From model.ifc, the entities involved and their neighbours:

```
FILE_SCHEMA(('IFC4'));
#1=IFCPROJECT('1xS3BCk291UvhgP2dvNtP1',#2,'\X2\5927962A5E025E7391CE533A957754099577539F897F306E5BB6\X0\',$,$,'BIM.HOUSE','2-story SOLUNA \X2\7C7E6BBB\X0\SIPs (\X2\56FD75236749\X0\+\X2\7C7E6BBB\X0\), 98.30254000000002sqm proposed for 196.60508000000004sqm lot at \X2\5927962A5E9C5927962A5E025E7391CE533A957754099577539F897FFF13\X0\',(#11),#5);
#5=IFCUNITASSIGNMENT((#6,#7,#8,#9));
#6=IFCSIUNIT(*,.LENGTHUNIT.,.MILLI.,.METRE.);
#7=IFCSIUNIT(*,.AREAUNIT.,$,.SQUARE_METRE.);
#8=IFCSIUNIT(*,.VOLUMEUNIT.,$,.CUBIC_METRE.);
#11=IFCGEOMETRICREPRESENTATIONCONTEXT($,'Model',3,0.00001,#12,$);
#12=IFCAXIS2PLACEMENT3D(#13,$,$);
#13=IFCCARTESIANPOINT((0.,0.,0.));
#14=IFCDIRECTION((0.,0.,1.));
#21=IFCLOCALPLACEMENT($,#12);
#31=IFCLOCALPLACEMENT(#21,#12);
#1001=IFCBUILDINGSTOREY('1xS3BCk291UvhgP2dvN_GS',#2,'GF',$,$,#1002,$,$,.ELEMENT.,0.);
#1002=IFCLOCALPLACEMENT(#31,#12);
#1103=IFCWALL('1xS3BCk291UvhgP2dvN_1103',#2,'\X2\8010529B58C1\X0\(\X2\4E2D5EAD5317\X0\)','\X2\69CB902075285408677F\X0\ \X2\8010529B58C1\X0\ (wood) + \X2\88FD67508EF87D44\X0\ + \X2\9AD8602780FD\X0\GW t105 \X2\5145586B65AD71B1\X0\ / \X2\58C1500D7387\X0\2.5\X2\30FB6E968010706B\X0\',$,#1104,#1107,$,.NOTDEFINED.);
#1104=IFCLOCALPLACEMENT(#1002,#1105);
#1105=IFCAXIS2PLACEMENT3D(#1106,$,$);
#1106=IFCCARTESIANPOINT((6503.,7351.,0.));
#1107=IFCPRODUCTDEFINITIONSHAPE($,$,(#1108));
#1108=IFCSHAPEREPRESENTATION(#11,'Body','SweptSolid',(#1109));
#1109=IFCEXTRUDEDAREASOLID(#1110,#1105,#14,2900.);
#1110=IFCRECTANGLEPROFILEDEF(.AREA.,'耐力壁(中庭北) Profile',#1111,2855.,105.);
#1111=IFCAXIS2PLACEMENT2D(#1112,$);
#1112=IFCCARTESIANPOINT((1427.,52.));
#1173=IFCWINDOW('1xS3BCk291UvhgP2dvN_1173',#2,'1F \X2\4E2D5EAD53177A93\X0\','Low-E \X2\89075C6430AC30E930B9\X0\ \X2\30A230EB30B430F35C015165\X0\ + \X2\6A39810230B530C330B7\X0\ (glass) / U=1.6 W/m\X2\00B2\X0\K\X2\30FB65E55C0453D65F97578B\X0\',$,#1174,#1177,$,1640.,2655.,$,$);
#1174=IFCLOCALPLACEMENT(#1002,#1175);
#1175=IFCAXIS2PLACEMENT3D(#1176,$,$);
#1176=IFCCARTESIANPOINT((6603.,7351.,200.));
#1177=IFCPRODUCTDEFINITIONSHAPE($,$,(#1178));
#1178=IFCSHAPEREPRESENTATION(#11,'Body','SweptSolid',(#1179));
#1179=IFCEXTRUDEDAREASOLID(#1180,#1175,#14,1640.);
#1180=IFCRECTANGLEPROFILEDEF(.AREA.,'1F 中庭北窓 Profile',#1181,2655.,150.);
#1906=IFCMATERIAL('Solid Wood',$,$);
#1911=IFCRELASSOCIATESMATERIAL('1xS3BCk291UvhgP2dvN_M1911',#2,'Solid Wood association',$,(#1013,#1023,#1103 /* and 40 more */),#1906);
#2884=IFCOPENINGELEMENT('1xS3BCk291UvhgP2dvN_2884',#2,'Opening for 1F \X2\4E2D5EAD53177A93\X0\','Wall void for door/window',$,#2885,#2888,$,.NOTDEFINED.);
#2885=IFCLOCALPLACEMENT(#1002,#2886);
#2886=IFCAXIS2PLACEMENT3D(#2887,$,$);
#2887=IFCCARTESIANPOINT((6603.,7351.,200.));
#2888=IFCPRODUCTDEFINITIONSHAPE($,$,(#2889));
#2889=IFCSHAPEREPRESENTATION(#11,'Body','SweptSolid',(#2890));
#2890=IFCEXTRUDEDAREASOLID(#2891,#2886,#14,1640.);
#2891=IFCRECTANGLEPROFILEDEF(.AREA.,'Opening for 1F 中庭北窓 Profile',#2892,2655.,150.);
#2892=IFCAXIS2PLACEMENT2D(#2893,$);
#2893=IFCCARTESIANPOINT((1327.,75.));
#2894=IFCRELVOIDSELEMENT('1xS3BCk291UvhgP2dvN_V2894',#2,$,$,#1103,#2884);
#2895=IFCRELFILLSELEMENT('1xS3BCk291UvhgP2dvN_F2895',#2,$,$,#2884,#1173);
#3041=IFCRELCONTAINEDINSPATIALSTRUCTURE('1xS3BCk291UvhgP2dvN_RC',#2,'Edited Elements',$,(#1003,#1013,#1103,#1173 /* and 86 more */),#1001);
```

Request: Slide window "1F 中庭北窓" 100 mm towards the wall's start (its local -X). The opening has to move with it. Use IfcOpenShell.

```python
import ifcopenshell
import ifcopenshell.api.geometry
import ifcopenshell.util.placement
import ifcopenshell.util.unit

model = ifcopenshell.open("model.ifc")
unit_scale = ifcopenshell.util.unit.calculate_unit_scale(model)

window = model.by_guid("1xS3BCk291UvhgP2dvN_1173")
opening = window.FillsVoids[0].RelatingOpeningElement
wall = opening.VoidsElements[0].RelatingBuildingElement

wall_matrix = ifcopenshell.util.placement.get_local_placement(wall.ObjectPlacement)
shift = wall_matrix[:3, 0] * -0.1 / unit_scale
before = ifcopenshell.util.placement.get_local_placement(window.ObjectPlacement)[:3, 3].copy()

# The window is not placed relative to its opening, so move both.
for product in (opening, window):
    matrix = ifcopenshell.util.placement.get_local_placement(product.ObjectPlacement)
    matrix[:3, 3] += shift
    ifcopenshell.api.geometry.edit_object_placement(model, product=product, matrix=matrix, is_si=False)

after = ifcopenshell.util.placement.get_local_placement(window.ObjectPlacement)[:3, 3]
print("window moved by", (after - before).round(3) + 0.0)

model.write("model_v2.ifc")
```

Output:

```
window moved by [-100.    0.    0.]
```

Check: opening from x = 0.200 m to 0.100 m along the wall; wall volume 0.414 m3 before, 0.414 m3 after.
